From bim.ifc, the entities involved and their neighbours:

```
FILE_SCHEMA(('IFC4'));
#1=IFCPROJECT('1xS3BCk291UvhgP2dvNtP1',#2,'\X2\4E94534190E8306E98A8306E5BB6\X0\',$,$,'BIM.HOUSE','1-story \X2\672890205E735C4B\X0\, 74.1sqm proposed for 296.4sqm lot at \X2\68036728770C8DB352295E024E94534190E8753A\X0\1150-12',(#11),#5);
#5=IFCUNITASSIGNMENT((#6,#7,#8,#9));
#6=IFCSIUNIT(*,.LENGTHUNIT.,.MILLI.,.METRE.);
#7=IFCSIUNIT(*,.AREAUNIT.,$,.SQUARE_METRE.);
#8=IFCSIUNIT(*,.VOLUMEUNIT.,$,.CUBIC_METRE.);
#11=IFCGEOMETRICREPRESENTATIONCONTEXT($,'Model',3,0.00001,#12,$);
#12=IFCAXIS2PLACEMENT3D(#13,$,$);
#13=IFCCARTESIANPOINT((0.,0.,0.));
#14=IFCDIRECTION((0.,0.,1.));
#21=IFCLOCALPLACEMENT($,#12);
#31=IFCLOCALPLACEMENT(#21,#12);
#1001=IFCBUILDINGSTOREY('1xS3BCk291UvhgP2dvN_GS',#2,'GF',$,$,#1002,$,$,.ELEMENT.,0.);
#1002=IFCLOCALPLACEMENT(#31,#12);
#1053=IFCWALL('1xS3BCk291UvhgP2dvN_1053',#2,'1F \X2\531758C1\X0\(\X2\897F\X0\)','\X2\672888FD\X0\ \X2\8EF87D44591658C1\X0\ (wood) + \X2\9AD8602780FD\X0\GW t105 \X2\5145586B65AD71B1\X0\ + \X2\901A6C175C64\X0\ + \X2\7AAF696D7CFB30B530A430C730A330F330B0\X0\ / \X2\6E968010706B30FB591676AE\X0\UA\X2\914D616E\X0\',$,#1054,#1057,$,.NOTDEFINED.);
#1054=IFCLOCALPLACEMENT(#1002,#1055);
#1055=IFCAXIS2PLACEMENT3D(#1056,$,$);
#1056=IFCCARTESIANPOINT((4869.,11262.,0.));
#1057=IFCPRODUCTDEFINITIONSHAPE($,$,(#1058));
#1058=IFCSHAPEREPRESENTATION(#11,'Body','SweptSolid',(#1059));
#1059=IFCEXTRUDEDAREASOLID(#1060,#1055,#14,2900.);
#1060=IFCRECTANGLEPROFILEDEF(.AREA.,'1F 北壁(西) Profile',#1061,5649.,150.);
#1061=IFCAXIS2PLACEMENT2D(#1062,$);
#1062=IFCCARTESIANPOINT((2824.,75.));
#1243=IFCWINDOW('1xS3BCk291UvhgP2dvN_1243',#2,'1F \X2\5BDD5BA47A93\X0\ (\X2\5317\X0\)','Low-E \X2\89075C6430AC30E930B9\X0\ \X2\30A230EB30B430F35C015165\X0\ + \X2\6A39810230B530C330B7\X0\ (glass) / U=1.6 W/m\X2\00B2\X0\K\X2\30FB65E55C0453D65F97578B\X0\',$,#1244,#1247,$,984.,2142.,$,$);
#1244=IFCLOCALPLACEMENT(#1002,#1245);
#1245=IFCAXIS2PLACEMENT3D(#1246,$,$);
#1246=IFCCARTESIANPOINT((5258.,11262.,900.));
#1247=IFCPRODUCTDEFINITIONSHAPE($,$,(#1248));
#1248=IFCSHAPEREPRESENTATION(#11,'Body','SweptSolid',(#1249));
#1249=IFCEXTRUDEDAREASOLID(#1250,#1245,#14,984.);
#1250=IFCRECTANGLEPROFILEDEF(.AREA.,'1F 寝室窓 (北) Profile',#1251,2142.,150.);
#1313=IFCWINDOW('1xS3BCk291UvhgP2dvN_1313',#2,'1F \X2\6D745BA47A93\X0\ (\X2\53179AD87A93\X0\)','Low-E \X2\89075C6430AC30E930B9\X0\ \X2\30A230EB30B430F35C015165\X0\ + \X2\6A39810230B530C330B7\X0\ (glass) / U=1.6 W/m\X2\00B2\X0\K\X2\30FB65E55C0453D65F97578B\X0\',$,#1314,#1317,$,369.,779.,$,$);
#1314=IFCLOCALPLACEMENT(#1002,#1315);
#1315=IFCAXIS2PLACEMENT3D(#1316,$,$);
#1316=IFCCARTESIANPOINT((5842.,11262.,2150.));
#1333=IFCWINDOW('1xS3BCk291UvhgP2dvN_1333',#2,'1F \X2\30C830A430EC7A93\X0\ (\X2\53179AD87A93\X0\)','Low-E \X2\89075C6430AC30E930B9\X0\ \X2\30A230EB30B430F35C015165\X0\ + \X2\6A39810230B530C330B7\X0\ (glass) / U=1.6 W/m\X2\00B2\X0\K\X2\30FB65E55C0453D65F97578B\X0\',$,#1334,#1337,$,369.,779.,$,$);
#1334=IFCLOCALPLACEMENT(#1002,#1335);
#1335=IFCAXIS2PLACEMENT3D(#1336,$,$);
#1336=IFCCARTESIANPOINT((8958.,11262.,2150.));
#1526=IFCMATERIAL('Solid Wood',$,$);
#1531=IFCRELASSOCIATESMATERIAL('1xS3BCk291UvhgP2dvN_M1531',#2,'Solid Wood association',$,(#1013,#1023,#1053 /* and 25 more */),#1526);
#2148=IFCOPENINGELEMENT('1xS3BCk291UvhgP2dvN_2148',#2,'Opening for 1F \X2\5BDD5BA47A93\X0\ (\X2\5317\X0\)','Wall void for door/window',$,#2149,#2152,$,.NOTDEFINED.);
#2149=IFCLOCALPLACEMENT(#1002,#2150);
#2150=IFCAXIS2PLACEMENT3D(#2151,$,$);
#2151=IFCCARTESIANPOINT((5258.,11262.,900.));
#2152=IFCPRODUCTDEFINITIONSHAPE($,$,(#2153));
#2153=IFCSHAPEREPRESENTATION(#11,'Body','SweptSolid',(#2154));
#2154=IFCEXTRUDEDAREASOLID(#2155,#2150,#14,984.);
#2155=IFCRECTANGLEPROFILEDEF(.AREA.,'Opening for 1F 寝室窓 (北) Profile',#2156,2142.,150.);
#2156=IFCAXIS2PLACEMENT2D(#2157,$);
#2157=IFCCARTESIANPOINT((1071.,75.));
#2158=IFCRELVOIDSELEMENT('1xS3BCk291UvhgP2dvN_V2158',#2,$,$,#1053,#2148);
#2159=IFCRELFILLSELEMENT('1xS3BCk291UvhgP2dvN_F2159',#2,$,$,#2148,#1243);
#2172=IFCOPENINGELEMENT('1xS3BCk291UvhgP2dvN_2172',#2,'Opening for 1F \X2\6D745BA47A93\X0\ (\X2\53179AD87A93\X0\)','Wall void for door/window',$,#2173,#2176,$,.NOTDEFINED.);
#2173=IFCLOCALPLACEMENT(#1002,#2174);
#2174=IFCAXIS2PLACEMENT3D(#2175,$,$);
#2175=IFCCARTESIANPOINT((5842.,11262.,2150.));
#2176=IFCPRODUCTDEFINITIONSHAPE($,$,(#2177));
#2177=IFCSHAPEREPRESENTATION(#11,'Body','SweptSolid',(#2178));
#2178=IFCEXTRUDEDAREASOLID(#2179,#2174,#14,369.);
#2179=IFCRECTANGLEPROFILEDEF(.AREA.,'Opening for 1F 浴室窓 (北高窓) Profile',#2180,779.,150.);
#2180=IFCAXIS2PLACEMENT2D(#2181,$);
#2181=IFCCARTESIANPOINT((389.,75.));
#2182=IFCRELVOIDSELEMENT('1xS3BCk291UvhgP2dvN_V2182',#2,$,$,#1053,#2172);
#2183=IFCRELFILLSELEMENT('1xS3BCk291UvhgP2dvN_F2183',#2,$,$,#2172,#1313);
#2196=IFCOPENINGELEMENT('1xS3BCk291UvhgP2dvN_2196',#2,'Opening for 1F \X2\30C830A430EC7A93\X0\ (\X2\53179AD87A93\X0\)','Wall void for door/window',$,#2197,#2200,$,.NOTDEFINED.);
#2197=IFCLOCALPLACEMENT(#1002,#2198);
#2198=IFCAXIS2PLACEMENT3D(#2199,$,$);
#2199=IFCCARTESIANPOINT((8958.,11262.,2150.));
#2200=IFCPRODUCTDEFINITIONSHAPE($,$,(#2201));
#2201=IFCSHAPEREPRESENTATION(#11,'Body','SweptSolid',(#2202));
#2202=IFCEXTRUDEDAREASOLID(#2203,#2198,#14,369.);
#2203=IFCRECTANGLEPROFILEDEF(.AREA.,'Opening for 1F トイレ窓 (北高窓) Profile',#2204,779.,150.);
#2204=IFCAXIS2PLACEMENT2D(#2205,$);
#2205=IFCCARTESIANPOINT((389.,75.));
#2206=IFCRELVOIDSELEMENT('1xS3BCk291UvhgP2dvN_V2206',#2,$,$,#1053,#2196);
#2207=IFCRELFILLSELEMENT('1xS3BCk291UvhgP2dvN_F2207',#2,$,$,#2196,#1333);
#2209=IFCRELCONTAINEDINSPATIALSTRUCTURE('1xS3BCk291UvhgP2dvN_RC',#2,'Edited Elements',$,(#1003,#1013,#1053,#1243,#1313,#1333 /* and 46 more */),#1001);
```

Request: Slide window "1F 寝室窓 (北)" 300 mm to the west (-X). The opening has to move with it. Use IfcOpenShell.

```python
import ifcopenshell
import ifcopenshell.api.geometry
import ifcopenshell.util.placement
import ifcopenshell.util.unit

model = ifcopenshell.open("bim.ifc")
unit_scale = ifcopenshell.util.unit.calculate_unit_scale(model)

window = model.by_id(1243)
opening = window.FillsVoids[0].RelatingOpeningElement
wall = opening.VoidsElements[0].RelatingBuildingElement

wall_matrix = ifcopenshell.util.placement.get_local_placement(wall.ObjectPlacement)
shift = wall_matrix[:3, 0] * -0.3 / unit_scale
before = ifcopenshell.util.placement.get_local_placement(window.ObjectPlacement)[:3, 3].copy()

# The window is not placed relative to its opening, so move both.
for product in (opening, window):
    matrix = ifcopenshell.util.placement.get_local_placement(product.ObjectPlacement)
    matrix[:3, 3] += shift
    ifcopenshell.api.geometry.edit_object_placement(model, product=product, matrix=matrix, is_si=False)

after = ifcopenshell.util.placement.get_local_placement(window.ObjectPlacement)[:3, 3]
print("window moved by", (after - before).round(3) + 0.0)

model.write("bim_edited.ifc")
```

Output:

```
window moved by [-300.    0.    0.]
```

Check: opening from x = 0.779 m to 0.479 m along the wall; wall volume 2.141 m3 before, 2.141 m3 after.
